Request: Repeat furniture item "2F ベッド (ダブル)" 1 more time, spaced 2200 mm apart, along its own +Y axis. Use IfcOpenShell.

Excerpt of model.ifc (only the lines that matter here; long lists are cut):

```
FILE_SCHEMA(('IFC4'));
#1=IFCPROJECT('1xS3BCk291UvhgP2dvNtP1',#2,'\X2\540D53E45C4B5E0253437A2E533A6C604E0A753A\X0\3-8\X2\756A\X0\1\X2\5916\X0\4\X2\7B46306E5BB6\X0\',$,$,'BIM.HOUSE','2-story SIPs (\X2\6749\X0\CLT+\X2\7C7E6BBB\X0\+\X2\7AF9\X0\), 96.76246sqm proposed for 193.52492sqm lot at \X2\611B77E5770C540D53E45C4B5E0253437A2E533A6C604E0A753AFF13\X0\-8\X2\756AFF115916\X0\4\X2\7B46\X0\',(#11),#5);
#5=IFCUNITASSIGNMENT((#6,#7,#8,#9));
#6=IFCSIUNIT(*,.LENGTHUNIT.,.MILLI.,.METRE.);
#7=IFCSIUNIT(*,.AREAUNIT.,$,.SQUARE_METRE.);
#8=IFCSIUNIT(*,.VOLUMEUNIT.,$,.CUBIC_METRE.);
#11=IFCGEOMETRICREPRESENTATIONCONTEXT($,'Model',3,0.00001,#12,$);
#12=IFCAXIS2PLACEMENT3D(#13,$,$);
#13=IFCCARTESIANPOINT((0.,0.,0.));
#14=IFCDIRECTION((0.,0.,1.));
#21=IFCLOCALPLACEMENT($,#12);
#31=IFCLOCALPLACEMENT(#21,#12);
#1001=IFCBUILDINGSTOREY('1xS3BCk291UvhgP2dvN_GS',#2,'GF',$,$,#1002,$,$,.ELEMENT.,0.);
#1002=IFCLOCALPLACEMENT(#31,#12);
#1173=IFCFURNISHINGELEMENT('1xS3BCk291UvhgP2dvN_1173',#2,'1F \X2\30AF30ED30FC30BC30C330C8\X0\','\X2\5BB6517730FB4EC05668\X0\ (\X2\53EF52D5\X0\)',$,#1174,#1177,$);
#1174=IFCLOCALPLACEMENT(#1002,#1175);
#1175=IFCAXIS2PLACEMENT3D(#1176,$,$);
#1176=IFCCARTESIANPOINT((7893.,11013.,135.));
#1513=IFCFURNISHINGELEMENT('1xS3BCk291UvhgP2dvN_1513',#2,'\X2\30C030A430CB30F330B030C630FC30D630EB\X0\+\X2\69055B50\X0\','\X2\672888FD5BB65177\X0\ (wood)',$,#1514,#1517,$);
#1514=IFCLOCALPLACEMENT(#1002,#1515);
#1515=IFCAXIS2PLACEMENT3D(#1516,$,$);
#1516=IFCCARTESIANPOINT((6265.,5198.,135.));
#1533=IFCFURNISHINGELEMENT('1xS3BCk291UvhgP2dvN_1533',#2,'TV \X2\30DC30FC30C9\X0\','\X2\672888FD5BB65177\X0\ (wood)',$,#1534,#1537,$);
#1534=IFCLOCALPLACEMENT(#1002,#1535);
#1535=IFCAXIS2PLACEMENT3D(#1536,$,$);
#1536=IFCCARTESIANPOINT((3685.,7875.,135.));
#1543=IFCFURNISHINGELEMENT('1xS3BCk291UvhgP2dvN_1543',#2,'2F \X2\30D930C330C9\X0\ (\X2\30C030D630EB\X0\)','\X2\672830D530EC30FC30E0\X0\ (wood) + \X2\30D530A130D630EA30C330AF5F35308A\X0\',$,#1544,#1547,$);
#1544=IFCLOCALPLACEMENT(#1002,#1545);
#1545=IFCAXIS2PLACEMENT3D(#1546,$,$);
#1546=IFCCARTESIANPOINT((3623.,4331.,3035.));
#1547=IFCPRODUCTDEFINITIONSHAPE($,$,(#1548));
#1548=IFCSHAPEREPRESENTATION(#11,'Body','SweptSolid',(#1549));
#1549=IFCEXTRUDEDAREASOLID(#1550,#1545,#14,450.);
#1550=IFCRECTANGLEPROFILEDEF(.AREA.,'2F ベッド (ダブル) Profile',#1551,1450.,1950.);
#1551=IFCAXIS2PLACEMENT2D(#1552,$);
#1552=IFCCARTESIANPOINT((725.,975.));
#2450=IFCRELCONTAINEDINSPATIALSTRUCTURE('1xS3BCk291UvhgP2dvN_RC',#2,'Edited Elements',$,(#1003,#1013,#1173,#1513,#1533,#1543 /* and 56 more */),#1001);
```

```python
import ifcopenshell
import ifcopenshell.api.geometry
import ifcopenshell.api.root
import ifcopenshell.util.element
import ifcopenshell.util.placement

model = ifcopenshell.open("model.ifc")


def reuse_history(source, copy):
    """copy_class also copies each property set's owner history, people and application; keep the originals."""
    for rel in copy.IsDefinedBy:
        if rel.is_a("IfcRelDefinesByProperties") and (history := rel.RelatingPropertyDefinition.OwnerHistory):
            rel.RelatingPropertyDefinition.OwnerHistory = source.OwnerHistory
            ifcopenshell.util.element.remove_deep2(model, history)


source = model.by_guid("1xS3BCk291UvhgP2dvN_1543")
base = ifcopenshell.util.placement.get_local_placement(source.ObjectPlacement)
step = base[:3, 1] * 2200.0

for i in range(1, 2):
    copy = ifcopenshell.api.root.copy_class(model, product=source)
    copy.Representation = ifcopenshell.util.element.copy_deep(
        model, source.Representation, exclude=["IfcGeometricRepresentationContext", "IfcRepresentationMap"]
    )
    reuse_history(source, copy)
    matrix = base.copy()
    matrix[:3, 3] += i * step
    print("added at", matrix[:3, 3].round(3) + 0.0)
    ifcopenshell.api.geometry.edit_object_placement(model, product=copy, matrix=matrix, is_si=False)

model.write("model_updated.ifc")
```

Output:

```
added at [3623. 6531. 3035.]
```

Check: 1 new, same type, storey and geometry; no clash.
